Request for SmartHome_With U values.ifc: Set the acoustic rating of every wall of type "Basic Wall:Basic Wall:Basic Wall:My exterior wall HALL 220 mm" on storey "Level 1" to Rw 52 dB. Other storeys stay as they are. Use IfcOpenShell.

First a look at what the model holds.

```python
import ifcopenshell
import ifcopenshell.util.element

model = ifcopenshell.open("SmartHome_With U values.ifc")
print(model.schema)
storey = next(s for s in model.by_type("IfcBuildingStorey") if s.Name == "Level 1")
walls = [e for e in ifcopenshell.util.element.get_decomposition(storey) if e.is_a("IfcWall")]
seen = {}
for e in walls:
    element_type = ifcopenshell.util.element.get_type(e)
    key = (element_type.Name if element_type != e and element_type else None, ifcopenshell.util.element.get_pset(e, "Pset_WallCommon", "AcousticRating"))
    seen[key] = seen.get(key, 0) + 1
for (name, value), count in sorted(seen.items(), key=str):
    print(count, "x", name, "|", value)
```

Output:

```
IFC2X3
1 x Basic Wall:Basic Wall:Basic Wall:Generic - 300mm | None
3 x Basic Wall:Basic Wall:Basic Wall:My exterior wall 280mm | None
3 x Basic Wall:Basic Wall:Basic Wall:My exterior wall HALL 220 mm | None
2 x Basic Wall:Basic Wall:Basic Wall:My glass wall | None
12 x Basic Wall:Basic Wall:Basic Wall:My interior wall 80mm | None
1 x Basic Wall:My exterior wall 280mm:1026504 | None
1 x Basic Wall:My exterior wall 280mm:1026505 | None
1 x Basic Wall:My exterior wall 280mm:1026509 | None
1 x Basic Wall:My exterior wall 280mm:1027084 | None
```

```python
import ifcopenshell
import ifcopenshell.api.pset
import ifcopenshell.util.element

model = ifcopenshell.open("SmartHome_With U values.ifc")

storey = next(s for s in model.by_type("IfcBuildingStorey") if s.Name == "Level 1")
walls = [e for e in ifcopenshell.util.element.get_decomposition(storey) if e.is_a("IfcWall")]

count = 0
for e in walls:
    element_type = ifcopenshell.util.element.get_type(e)
    if element_type in (None, e) or element_type.Name != "Basic Wall:Basic Wall:Basic Wall:My exterior wall HALL 220 mm":
        continue
    # add_pset returns the element's existing set when there is one.
    pset = ifcopenshell.api.pset.add_pset(model, product=e, name="Pset_WallCommon")
    ifcopenshell.api.pset.edit_pset(model, pset=pset, properties={"AcousticRating": "Rw 52 dB"})
    count += 1

print(count, "walls updated")

model.write("SmartHome_With U values_updated.ifc")
```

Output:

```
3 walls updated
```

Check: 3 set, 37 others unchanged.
